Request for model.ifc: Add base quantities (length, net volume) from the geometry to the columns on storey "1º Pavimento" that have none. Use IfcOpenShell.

First a look at what the model holds.

```python
import ifcopenshell
import ifcopenshell.util.element
import ifcopenshell.util.unit

model = ifcopenshell.open("model.ifc")
print(model.schema)
for unit_type in ("LENGTHUNIT", "AREAUNIT", "VOLUMEUNIT"):
    print(unit_type, ifcopenshell.util.unit.calculate_unit_scale(model, unit_type))
storey = next(s for s in model.by_type("IfcBuildingStorey") if s.Name == "1º Pavimento")
columns = [e for e in ifcopenshell.util.element.get_decomposition(storey) if e.is_a("IfcColumn")]
for e in sorted(columns, key=lambda e: e.id()):
    print(e.id(), e.is_a(), e.Name, list(ifcopenshell.util.element.get_psets(e, qtos_only=True)), sep=" | ")
```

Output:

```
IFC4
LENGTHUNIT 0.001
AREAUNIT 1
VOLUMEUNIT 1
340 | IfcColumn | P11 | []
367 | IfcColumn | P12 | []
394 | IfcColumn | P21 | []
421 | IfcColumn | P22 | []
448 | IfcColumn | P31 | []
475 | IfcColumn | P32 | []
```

```python
import ifcopenshell
import ifcopenshell.api.pset
import ifcopenshell.geom
import ifcopenshell.util.element
import ifcopenshell.util.shape
import ifcopenshell.util.unit

model = ifcopenshell.open("model.ifc")
unit_scale = ifcopenshell.util.unit.calculate_unit_scale(model)
volume_scale = ifcopenshell.util.unit.calculate_unit_scale(model, "VOLUMEUNIT")
settings = ifcopenshell.geom.settings()

storey = next(s for s in model.by_type("IfcBuildingStorey") if s.Name == "1º Pavimento")
columns = [e for e in ifcopenshell.util.element.get_decomposition(storey) if e.is_a("IfcColumn")]

for e in sorted(columns, key=lambda e: e.id()):
    if ifcopenshell.util.element.get_psets(e, qtos_only=True, should_inherit=False):
        continue
    # Geometry comes back in metres, in the element's own axes.
    shape = ifcopenshell.geom.create_shape(settings, e)
    values = {
        "Length": ifcopenshell.util.shape.get_z(shape.geometry) / unit_scale,
        "NetVolume": ifcopenshell.util.shape.get_volume(shape.geometry) / volume_scale,
    }
    qto = ifcopenshell.api.pset.add_qto(model, product=e, name="Qto_ColumnBaseQuantities")
    ifcopenshell.api.pset.edit_qto(model, qto=qto, properties=values)
    print(e.id(), {k: round(v, 3) for k, v in values.items()})

model.write("model_v2.ifc")
```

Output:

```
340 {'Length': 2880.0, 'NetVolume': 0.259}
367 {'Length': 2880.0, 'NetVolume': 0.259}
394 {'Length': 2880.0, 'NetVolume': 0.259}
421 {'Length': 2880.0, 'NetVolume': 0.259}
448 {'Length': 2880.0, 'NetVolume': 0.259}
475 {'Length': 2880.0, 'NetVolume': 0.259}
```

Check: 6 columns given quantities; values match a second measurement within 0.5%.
